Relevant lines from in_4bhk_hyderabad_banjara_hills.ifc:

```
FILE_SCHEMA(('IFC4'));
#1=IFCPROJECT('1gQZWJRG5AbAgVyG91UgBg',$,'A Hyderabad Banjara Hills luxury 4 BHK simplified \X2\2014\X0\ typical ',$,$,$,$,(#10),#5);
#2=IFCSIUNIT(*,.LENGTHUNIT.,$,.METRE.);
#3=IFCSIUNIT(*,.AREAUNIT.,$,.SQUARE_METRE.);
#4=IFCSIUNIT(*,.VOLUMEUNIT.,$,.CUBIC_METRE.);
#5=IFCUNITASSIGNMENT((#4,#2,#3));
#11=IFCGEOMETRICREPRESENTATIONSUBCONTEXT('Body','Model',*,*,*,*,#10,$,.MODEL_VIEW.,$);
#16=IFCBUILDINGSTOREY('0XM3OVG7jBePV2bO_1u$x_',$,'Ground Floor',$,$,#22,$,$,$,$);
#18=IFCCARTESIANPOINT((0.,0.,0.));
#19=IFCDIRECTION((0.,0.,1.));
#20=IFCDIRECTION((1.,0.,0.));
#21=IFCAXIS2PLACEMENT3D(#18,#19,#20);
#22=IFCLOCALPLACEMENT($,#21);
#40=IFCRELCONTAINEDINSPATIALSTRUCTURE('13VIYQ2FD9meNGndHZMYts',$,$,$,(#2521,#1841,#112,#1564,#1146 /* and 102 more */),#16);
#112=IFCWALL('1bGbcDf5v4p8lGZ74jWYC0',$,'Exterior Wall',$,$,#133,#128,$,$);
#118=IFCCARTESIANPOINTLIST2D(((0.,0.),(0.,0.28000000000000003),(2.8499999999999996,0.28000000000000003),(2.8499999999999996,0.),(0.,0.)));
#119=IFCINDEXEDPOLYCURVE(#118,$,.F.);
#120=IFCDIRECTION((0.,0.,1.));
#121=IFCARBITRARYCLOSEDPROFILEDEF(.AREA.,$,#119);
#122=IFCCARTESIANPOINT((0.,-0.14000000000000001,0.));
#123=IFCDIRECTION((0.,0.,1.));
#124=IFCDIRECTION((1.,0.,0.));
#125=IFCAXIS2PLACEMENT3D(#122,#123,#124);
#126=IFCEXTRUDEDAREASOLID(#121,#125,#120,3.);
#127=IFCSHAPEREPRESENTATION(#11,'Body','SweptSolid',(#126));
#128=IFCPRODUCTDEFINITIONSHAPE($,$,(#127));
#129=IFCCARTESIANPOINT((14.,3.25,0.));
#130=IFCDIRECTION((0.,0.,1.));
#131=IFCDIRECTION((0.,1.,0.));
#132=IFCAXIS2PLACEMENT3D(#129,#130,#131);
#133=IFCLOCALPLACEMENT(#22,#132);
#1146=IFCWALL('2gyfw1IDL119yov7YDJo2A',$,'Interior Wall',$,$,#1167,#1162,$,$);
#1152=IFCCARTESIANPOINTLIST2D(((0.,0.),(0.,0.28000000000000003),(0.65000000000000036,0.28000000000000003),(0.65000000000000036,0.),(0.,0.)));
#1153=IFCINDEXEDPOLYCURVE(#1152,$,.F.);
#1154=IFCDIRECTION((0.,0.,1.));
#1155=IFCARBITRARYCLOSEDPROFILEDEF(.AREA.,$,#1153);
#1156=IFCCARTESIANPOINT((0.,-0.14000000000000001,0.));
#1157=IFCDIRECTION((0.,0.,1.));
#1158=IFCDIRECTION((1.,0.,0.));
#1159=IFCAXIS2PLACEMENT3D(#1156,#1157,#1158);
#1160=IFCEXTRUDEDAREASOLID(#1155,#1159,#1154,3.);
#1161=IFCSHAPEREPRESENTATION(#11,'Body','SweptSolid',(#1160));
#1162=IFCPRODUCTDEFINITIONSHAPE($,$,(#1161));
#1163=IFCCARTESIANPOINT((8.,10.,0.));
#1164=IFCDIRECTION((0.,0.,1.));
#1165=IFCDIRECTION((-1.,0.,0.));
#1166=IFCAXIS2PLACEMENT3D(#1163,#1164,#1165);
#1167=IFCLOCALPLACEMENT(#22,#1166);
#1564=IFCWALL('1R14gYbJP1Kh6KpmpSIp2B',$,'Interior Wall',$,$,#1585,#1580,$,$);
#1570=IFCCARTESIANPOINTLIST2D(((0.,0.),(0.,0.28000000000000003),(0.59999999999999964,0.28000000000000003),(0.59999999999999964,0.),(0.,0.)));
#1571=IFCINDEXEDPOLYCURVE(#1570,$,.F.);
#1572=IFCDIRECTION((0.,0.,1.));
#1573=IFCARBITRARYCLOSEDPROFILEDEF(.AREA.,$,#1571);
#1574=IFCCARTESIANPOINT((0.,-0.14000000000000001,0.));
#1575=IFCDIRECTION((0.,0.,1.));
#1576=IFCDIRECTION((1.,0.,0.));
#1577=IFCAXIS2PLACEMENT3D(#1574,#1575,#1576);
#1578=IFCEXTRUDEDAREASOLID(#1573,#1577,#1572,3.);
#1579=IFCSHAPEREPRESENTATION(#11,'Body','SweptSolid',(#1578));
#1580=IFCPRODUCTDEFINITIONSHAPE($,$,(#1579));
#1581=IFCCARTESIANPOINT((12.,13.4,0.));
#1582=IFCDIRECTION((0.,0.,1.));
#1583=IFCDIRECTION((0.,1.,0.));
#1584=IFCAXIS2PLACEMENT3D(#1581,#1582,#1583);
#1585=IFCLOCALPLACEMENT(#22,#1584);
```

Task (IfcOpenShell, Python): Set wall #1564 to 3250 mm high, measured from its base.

```python
import ifcopenshell
import ifcopenshell.geom
import ifcopenshell.util.representation
import ifcopenshell.util.shape
import ifcopenshell.util.unit

model = ifcopenshell.open("in_4bhk_hyderabad_banjara_hills.ifc")
unit_scale = ifcopenshell.util.unit.calculate_unit_scale(model)
settings = ifcopenshell.geom.settings()


def volume(element):
    """Net volume in cubic metres, openings subtracted."""
    shape = ifcopenshell.geom.create_shape(settings, element)
    return ifcopenshell.util.shape.get_volume(shape.geometry)


wall = model.by_id(1564)
before = volume(wall)

body = ifcopenshell.util.representation.get_representation(wall, "Model", "Body")
solid = body.Items[0]
old_height = solid.Depth
solid.Depth = 3.25 / unit_scale
after = volume(wall)

print(f"height {old_height:g} -> {solid.Depth:g}, volume {before:.3f} -> {after:.3f} m3")

model.write("in_4bhk_hyderabad_banjara_hills_updated.ifc")
```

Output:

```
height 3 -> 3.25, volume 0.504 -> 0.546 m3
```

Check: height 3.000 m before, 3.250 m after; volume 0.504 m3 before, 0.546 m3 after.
